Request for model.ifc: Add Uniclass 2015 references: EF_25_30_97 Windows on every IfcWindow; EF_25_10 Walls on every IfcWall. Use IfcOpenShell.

First a look at what the model holds.

```python
import ifcopenshell

model = ifcopenshell.open("model.ifc")
print(model.schema)
print("classifications:", [c.Name for c in model.by_type("IfcClassification")])
for ifc_class in ("IfcDoor", "IfcRoof", "IfcStair", "IfcWall", "IfcWindow"):
    print(ifc_class, len(model.by_type(ifc_class)))
```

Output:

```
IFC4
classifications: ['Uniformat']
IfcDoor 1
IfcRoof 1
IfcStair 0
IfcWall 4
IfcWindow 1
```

```python
import ifcopenshell
import ifcopenshell.api.classification

model = ifcopenshell.open("model.ifc")

system = ifcopenshell.api.classification.add_classification(model, classification="Uniclass 2015")

codes = {
    "IfcWindow": ("EF_25_30_97", "Windows"),
    "IfcWall": ("EF_25_10", "Walls"),
}
for ifc_class, (code, name) in codes.items():
    products = model.by_type(ifc_class)
    ifcopenshell.api.classification.add_reference(
        model, products=products, classification=system, identification=code, name=name
    )
    print(code, len(products))

model.write("model_edited.ifc")
```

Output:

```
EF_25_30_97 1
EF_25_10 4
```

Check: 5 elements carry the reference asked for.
